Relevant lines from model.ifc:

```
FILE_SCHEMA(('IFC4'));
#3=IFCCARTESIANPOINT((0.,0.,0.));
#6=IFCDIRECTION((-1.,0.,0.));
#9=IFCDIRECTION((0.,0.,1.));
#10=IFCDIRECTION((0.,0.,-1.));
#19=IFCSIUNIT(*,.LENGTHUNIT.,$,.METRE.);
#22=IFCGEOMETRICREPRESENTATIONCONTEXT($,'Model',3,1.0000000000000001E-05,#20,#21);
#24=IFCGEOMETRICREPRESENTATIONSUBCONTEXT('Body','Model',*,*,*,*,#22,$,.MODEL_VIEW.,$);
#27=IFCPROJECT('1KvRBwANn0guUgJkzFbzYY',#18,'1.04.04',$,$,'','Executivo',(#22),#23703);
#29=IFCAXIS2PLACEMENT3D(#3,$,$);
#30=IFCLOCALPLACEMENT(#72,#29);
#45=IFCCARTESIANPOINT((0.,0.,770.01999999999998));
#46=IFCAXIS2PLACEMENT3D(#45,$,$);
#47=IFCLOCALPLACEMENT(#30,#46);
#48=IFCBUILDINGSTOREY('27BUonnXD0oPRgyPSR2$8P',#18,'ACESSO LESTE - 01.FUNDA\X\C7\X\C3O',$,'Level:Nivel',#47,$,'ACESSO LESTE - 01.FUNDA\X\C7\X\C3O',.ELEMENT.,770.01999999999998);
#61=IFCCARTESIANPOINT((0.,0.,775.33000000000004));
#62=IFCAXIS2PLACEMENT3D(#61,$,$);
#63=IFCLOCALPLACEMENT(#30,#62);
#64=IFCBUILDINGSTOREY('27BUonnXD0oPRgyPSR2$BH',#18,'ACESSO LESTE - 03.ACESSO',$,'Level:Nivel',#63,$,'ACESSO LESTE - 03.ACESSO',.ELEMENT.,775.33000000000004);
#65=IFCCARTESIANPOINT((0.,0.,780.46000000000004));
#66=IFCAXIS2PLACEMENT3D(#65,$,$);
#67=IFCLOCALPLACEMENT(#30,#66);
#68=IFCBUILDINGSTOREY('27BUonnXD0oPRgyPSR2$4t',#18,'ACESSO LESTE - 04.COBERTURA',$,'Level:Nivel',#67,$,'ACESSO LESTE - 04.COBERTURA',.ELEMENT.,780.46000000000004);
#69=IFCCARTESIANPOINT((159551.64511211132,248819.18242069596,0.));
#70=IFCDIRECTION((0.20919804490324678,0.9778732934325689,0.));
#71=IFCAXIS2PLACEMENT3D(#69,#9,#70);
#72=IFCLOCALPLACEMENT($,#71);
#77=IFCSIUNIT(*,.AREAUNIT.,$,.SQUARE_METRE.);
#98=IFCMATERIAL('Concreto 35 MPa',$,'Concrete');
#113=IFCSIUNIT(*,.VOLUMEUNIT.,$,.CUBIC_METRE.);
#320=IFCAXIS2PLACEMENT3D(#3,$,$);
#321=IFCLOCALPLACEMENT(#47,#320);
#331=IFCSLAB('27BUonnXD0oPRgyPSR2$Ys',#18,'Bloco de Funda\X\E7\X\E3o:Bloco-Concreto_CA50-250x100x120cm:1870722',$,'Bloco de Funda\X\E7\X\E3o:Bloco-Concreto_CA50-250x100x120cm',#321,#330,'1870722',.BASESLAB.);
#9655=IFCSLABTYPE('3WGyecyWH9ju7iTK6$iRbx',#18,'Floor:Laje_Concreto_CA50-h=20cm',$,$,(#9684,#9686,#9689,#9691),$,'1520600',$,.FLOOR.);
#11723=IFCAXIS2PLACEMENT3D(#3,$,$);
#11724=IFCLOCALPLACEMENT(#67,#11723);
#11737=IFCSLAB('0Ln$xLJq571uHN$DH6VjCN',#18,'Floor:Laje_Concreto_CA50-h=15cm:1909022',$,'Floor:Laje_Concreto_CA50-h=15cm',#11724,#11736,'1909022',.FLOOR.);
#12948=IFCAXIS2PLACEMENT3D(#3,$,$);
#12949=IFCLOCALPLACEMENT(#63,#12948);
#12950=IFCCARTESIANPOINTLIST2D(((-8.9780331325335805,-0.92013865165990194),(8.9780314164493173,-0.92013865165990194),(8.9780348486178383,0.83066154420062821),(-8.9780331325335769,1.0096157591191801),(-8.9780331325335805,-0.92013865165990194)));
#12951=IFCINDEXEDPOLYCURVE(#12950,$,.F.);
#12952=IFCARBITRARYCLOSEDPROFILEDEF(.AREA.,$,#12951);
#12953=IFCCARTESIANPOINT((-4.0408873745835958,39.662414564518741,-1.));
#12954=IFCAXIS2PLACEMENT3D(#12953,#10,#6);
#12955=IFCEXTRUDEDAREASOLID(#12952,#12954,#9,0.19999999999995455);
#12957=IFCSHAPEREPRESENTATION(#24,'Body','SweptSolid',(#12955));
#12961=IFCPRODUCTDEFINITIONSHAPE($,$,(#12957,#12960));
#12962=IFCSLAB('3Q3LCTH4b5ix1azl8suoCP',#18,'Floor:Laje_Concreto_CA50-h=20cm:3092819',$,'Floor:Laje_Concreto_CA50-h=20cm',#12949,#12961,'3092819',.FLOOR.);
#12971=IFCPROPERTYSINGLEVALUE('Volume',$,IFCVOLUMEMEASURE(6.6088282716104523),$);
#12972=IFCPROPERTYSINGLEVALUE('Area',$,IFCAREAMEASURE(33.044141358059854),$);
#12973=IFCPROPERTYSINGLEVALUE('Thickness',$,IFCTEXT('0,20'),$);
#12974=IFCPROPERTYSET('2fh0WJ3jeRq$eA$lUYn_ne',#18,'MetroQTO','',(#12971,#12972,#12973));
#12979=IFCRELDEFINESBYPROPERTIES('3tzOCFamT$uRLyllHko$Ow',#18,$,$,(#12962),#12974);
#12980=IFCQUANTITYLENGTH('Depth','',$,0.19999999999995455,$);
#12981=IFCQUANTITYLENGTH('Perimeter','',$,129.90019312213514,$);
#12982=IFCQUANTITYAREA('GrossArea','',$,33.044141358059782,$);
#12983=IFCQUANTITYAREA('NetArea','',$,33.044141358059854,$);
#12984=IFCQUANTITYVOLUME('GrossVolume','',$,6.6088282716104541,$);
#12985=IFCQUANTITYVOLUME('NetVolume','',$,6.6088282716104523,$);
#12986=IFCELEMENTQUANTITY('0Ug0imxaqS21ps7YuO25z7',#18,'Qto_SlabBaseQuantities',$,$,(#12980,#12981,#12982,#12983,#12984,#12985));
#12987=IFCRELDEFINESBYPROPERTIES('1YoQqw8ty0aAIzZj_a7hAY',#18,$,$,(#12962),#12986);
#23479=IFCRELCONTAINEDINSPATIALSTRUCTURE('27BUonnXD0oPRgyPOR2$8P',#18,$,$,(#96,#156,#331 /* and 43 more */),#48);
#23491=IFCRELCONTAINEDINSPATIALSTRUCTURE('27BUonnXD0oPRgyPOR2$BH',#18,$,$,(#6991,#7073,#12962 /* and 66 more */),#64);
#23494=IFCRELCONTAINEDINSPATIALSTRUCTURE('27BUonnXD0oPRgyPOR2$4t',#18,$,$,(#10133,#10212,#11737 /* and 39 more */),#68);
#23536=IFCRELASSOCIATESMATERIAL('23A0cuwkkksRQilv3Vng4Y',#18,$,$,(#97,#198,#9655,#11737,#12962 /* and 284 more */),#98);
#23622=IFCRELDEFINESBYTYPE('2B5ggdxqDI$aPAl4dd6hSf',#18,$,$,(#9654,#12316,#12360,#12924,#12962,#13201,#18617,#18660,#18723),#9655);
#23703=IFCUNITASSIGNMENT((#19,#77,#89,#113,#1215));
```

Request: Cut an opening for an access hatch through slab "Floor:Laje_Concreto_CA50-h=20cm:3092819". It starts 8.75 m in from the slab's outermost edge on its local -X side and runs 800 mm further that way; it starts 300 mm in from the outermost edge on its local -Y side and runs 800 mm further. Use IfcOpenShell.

```python
import numpy as np
import ifcopenshell
import ifcopenshell.api.feature
import ifcopenshell.api.geometry
import ifcopenshell.api.pset
import ifcopenshell.api.root
import ifcopenshell.geom
import ifcopenshell.util.element
import ifcopenshell.util.placement
import ifcopenshell.util.representation
import ifcopenshell.util.shape
import ifcopenshell.util.unit

model = ifcopenshell.open("model.ifc")
unit_scale = ifcopenshell.util.unit.calculate_unit_scale(model)
area_scale = ifcopenshell.util.unit.calculate_unit_scale(model, "AREAUNIT")
volume_scale = ifcopenshell.util.unit.calculate_unit_scale(model, "VOLUMEUNIT")
settings = ifcopenshell.geom.settings()


def volume(element):
    """Net volume in cubic metres, openings subtracted."""
    shape = ifcopenshell.geom.create_shape(settings, element)
    return ifcopenshell.util.shape.get_volume(shape.geometry)


slab = model.by_id(12962)
before = volume(slab)

# Extent in the slab's own axes, in metres. The edges named are its -X and -Y sides.
slab_shape = ifcopenshell.geom.create_shape(settings, slab)
vertices = ifcopenshell.util.shape.get_vertices(slab_shape.geometry)
x_min, y_min, bottom = vertices.min(axis=0)
top = vertices[:, 2].max()

opening = ifcopenshell.api.root.create_entity(model, ifc_class="IfcOpeningElement", name="Access hatch opening", predefined_type="OPENING")
context = ifcopenshell.util.representation.get_context(model, "Model", "Body", "MODEL_VIEW")
width, depth = 0.8, 0.8
outline = [(0.0, 0.0), (width, 0.0), (width, depth), (0.0, depth), (0.0, 0.0)]
# Overshoot both faces by 50 mm so the cut is clean.
shape = ifcopenshell.api.geometry.add_slab_representation(
    model, context=context, depth=top - bottom + 0.1, polyline=outline
)
ifcopenshell.api.geometry.assign_representation(model, product=opening, representation=shape)

matrix = ifcopenshell.util.placement.get_local_placement(slab.ObjectPlacement)
matrix[:, 3] = matrix @ np.append(np.array([x_min + 8.75, y_min + 0.3, bottom - 0.05]) / unit_scale, 1.0)
ifcopenshell.api.geometry.edit_object_placement(model, product=opening, matrix=matrix, is_si=False)
ifcopenshell.api.feature.add_feature(model, feature=opening, element=slab)

after = volume(slab)

# Update the slab's stored quantities.
pset = model.by_id(ifcopenshell.util.element.get_pset(slab, "MetroQTO", should_inherit=False)["id"])
ifcopenshell.api.pset.edit_pset(model, pset=pset, properties={
    "Volume": model.create_entity("IfcVolumeMeasure", after / volume_scale),
    "Area": model.create_entity("IfcAreaMeasure", after / (top - bottom) / area_scale),
})
qto = model.by_id(ifcopenshell.util.element.get_pset(slab, "Qto_SlabBaseQuantities", should_inherit=False)["id"])
ifcopenshell.api.pset.edit_qto(model, qto=qto, properties={
    "NetArea": after / (top - bottom) / area_scale,
    "NetVolume": after / volume_scale,
})

print(f"slab volume {before:.3f} -> {after:.3f} m3")

model.write("model_updated.ifc")
```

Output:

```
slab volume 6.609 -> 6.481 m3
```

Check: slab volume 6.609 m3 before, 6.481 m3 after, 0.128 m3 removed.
